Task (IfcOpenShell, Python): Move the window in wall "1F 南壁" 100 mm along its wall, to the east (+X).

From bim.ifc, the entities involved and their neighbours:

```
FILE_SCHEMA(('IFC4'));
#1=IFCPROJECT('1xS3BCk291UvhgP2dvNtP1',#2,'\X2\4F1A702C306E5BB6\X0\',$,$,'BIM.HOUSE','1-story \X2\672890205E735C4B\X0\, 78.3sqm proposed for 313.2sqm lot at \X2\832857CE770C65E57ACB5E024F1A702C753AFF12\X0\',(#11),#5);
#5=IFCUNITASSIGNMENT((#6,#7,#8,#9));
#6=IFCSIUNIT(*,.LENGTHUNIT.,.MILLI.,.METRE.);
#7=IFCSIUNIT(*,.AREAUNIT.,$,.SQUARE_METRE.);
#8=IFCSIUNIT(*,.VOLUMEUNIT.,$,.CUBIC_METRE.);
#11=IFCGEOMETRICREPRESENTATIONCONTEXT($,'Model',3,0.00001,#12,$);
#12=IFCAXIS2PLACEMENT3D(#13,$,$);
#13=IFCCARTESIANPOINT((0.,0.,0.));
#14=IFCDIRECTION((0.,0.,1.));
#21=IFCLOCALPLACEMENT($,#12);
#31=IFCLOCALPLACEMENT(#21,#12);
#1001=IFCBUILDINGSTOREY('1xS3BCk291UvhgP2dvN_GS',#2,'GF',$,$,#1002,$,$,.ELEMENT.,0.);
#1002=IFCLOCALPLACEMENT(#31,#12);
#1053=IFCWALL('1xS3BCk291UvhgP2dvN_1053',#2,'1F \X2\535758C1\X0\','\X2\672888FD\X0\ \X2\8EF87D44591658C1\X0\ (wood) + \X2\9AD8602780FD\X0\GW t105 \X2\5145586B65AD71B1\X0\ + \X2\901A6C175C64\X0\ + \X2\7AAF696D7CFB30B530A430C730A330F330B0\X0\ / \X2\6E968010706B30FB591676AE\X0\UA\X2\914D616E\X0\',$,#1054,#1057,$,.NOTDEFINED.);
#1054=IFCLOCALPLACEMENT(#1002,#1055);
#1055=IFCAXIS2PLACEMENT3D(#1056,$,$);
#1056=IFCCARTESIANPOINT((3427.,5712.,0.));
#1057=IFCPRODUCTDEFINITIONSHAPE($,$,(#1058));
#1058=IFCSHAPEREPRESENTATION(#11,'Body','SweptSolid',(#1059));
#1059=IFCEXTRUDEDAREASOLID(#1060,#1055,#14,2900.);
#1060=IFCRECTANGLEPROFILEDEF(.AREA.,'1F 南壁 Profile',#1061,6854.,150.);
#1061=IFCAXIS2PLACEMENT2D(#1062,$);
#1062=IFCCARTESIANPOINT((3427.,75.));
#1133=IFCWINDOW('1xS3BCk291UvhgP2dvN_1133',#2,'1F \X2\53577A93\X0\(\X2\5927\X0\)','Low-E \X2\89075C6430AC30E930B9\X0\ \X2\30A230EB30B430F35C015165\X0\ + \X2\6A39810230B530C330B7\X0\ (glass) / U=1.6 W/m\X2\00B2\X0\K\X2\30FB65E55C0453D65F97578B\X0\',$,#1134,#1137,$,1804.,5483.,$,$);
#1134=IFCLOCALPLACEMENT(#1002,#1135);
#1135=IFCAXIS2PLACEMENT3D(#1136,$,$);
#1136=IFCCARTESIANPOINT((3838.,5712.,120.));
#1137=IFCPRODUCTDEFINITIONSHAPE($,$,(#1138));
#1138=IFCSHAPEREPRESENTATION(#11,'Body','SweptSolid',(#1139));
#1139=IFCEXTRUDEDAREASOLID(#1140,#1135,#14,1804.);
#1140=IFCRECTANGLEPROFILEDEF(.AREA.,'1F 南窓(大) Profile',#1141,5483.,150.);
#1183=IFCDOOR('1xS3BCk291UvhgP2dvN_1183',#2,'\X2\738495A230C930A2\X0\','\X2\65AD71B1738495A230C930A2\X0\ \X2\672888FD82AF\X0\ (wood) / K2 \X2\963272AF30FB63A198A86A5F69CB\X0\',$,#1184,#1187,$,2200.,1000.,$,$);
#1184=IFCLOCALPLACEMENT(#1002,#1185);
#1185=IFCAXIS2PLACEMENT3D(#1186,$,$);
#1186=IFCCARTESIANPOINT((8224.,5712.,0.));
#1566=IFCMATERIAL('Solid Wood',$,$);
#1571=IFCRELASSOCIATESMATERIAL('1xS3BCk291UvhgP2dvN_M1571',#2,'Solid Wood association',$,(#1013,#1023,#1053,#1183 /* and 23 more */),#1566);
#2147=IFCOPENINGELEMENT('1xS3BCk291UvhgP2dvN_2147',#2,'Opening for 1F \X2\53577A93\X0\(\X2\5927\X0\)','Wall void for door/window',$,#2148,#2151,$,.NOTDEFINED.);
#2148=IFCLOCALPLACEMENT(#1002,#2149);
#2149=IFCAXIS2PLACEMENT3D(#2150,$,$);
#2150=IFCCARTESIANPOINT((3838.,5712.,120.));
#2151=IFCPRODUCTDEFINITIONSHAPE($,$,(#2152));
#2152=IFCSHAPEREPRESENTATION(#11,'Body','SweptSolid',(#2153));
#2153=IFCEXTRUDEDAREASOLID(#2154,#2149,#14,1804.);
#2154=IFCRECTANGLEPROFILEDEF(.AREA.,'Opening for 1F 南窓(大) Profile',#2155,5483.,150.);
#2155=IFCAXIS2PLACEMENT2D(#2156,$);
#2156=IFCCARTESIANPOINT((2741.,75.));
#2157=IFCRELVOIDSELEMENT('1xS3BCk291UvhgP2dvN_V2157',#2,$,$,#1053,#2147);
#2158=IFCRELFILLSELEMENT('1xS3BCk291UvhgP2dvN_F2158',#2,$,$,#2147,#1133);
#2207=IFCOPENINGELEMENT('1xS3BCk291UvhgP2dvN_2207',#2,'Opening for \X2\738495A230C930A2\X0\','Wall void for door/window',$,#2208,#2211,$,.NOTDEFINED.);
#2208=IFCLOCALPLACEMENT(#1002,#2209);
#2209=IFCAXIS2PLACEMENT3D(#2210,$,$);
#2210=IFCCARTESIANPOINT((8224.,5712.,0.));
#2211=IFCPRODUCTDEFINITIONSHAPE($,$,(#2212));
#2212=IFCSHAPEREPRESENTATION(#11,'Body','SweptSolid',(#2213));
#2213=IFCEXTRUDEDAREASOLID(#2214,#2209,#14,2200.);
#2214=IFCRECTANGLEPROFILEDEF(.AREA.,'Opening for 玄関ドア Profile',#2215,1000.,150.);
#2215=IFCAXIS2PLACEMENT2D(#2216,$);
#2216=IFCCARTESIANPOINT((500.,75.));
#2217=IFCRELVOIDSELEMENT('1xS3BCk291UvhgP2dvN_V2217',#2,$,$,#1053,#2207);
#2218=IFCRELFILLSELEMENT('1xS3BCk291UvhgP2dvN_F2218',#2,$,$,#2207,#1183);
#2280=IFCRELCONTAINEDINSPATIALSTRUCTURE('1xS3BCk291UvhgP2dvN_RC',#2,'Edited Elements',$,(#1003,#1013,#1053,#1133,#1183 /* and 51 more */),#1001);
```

```python
import ifcopenshell
import ifcopenshell.api.geometry
import ifcopenshell.util.placement

model = ifcopenshell.open("bim.ifc")

window = model.by_id(1133)
opening = window.FillsVoids[0].RelatingOpeningElement
wall = opening.VoidsElements[0].RelatingBuildingElement

wall_matrix = ifcopenshell.util.placement.get_local_placement(wall.ObjectPlacement)
shift = wall_matrix[:3, 0] * 100.0
before = ifcopenshell.util.placement.get_local_placement(window.ObjectPlacement)[:3, 3].copy()

# The window is not placed relative to its opening, so move both.
for product in (opening, window):
    matrix = ifcopenshell.util.placement.get_local_placement(product.ObjectPlacement)
    matrix[:3, 3] += shift
    ifcopenshell.api.geometry.edit_object_placement(model, product=product, matrix=matrix, is_si=False)

after = ifcopenshell.util.placement.get_local_placement(window.ObjectPlacement)[:3, 3]
print("window moved by", (after - before).round(3) + 0.0)

model.write("bim_updated.ifc")
```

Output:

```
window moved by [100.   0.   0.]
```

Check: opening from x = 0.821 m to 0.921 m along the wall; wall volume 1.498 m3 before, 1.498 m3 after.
